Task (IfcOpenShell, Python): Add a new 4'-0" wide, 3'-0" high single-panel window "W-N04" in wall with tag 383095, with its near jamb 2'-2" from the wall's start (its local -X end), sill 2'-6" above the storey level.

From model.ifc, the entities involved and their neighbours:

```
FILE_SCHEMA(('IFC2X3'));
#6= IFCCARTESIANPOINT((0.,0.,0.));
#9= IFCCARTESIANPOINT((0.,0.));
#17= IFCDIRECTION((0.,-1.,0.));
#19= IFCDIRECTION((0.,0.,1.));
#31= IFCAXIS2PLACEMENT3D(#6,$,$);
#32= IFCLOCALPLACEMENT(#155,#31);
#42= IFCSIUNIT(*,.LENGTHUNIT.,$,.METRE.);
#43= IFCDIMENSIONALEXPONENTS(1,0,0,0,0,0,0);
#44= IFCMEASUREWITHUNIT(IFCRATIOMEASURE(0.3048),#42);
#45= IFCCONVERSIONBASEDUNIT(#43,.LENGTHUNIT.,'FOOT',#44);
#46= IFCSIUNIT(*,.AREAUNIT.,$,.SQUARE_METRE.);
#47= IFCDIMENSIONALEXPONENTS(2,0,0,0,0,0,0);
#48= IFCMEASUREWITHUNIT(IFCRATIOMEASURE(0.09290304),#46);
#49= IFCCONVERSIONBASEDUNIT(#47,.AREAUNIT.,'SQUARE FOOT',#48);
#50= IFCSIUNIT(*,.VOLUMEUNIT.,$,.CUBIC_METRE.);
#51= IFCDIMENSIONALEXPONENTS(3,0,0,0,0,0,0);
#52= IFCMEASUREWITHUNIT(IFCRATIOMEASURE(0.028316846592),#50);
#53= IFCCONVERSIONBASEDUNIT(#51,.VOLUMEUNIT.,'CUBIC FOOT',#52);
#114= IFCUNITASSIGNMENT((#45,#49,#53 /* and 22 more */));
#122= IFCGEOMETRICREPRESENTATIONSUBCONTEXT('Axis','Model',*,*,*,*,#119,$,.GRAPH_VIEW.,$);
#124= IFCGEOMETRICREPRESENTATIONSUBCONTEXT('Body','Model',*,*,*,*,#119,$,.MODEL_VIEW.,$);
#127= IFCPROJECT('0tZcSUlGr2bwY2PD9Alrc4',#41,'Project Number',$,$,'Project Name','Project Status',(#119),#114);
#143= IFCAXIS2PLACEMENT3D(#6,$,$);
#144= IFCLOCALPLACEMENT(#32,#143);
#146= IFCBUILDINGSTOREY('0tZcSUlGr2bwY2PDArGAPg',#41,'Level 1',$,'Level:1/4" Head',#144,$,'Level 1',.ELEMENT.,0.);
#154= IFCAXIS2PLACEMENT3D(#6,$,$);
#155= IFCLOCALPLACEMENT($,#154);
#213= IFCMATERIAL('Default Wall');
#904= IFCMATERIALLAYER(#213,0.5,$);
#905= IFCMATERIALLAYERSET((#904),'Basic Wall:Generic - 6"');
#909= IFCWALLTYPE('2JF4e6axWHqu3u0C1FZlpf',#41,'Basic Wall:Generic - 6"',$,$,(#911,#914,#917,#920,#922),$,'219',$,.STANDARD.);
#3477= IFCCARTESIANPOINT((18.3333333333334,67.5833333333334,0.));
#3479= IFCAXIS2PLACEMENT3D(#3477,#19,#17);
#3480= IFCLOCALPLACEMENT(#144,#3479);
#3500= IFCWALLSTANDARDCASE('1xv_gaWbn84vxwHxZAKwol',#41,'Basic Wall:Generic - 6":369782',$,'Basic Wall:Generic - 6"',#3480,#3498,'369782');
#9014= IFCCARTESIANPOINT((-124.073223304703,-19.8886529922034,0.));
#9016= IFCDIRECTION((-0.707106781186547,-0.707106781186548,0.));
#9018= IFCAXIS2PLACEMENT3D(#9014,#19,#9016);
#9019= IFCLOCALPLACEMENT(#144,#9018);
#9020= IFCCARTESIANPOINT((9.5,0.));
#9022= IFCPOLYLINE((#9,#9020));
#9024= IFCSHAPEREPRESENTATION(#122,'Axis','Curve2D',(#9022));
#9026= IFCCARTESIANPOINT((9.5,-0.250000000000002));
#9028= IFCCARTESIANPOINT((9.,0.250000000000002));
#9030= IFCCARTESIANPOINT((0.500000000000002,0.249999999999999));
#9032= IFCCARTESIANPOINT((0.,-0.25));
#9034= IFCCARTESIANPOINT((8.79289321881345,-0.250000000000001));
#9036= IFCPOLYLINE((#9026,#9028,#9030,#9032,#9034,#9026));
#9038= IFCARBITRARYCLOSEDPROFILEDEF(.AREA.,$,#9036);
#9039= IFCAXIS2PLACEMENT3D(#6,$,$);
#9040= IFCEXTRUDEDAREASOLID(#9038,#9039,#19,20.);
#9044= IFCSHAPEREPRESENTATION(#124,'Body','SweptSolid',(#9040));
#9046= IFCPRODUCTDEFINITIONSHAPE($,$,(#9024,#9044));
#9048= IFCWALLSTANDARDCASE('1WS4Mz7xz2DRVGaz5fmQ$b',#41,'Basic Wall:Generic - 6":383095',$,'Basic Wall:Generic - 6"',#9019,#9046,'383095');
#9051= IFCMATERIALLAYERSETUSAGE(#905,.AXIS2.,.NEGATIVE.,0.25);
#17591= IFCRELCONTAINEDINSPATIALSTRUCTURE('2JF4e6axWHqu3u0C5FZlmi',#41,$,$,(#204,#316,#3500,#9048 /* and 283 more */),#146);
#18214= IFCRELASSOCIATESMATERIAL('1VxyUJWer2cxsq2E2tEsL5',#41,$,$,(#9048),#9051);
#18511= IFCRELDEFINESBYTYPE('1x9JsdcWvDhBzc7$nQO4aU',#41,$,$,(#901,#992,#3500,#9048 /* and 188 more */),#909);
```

```python
import numpy as np
import ifcopenshell
import ifcopenshell.api.feature
import ifcopenshell.api.geometry
import ifcopenshell.api.root
import ifcopenshell.api.spatial
import ifcopenshell.api.type
import ifcopenshell.geom
import ifcopenshell.util.element
import ifcopenshell.util.placement
import ifcopenshell.util.representation
import ifcopenshell.util.shape
import ifcopenshell.util.unit

model = ifcopenshell.open("model.ifc")
unit_scale = ifcopenshell.util.unit.calculate_unit_scale(model)
settings = ifcopenshell.geom.settings()


def volume(element):
    """Net volume in cubic metres, openings subtracted."""
    shape = ifcopenshell.geom.create_shape(settings, element)
    return ifcopenshell.util.shape.get_volume(shape.geometry)


wall = model.by_guid("1WS4Mz7xz2DRVGaz5fmQ$b")
storey = ifcopenshell.util.element.get_container(wall, ifc_class="IfcBuildingStorey")
context = ifcopenshell.util.representation.get_context(model, "Model", "Body", "MODEL_VIEW")
before = volume(wall)

width, height, from_end, sill = 1.2192, 0.9144, 0.6604, 0.762  # metres

# The wall runs along its own X axis, and the end named is its -X end.
wall_shape = ifcopenshell.geom.create_shape(settings, wall)
x, y, z = ifcopenshell.util.shape.get_vertices(wall_shape.geometry).T
start = x.min() + from_end
face, thickness = float(y.min()), float(y.max() - y.min())
wall_matrix = ifcopenshell.util.placement.get_local_placement(wall.ObjectPlacement)
level = ifcopenshell.util.placement.get_local_placement(storey.ObjectPlacement)[2, 3]


def in_wall(x, y):
    """Placement at x, y metres in the wall's axes, at sill height."""
    matrix = wall_matrix.copy()
    matrix[:, 3] = wall_matrix @ np.array([x / unit_scale, y / unit_scale, 0.0, 1.0])
    matrix[2, 3] = level + sill / unit_scale
    return matrix


# Opening: a box that overshoots both wall faces by 50 mm.
opening = ifcopenshell.api.root.create_entity(model, ifc_class="IfcOpeningElement")
box = ifcopenshell.api.geometry.add_wall_representation(
    model, context=context, length=width, height=height, thickness=thickness + 0.1
)
ifcopenshell.api.geometry.assign_representation(model, product=opening, representation=box)
ifcopenshell.api.geometry.edit_object_placement(model, product=opening, matrix=in_wall(start, face - 0.05), is_si=False)
ifcopenshell.api.feature.add_feature(model, feature=opening, element=wall)

window = ifcopenshell.api.root.create_entity(model, ifc_class="IfcWindow", name="W-N04")
window.OverallWidth, window.OverallHeight = width / unit_scale, height / unit_scale
body = ifcopenshell.api.geometry.add_window_representation(
    model,
    context=context,
    overall_width=window.OverallWidth,
    overall_height=window.OverallHeight,
    partition_type="SINGLE_PANEL",
)
ifcopenshell.api.geometry.assign_representation(model, product=window, representation=body)
ifcopenshell.api.spatial.assign_container(model, products=[window], relating_structure=storey)
fills = ifcopenshell.api.feature.add_filling(model, opening=opening, element=window)
fills.OwnerHistory = window.OwnerHistory  # required in IFC2X3

# IFC2X3 keeps the operation on the window style.
style = ifcopenshell.api.root.create_entity(model, ifc_class="IfcWindowStyle", name="W-N04")
style.OperationType, style.ConstructionType = "SINGLE_PANEL", "NOTDEFINED"
style.ParameterTakesPrecedence = style.Sizeable = False
ifcopenshell.api.type.assign_type(model, related_objects=[window], relating_type=style)

# Centre the window in the wall's thickness.
ifcopenshell.api.geometry.edit_object_placement(model, product=window, matrix=in_wall(start, face), is_si=False)
window_shape = ifcopenshell.geom.create_shape(settings, window)
depth = ifcopenshell.util.shape.get_vertices(window_shape.geometry)[:, 1]
offset = face + thickness / 2 - (depth.min() + depth.max()) / 2
ifcopenshell.api.geometry.edit_object_placement(model, product=window, matrix=in_wall(start, offset), is_si=False)

after = volume(wall)

print(f"wall volume {before:.3f} -> {after:.3f} m3")

model.write("model-out.ifc")
```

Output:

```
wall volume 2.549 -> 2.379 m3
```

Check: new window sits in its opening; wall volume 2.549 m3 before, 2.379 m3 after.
